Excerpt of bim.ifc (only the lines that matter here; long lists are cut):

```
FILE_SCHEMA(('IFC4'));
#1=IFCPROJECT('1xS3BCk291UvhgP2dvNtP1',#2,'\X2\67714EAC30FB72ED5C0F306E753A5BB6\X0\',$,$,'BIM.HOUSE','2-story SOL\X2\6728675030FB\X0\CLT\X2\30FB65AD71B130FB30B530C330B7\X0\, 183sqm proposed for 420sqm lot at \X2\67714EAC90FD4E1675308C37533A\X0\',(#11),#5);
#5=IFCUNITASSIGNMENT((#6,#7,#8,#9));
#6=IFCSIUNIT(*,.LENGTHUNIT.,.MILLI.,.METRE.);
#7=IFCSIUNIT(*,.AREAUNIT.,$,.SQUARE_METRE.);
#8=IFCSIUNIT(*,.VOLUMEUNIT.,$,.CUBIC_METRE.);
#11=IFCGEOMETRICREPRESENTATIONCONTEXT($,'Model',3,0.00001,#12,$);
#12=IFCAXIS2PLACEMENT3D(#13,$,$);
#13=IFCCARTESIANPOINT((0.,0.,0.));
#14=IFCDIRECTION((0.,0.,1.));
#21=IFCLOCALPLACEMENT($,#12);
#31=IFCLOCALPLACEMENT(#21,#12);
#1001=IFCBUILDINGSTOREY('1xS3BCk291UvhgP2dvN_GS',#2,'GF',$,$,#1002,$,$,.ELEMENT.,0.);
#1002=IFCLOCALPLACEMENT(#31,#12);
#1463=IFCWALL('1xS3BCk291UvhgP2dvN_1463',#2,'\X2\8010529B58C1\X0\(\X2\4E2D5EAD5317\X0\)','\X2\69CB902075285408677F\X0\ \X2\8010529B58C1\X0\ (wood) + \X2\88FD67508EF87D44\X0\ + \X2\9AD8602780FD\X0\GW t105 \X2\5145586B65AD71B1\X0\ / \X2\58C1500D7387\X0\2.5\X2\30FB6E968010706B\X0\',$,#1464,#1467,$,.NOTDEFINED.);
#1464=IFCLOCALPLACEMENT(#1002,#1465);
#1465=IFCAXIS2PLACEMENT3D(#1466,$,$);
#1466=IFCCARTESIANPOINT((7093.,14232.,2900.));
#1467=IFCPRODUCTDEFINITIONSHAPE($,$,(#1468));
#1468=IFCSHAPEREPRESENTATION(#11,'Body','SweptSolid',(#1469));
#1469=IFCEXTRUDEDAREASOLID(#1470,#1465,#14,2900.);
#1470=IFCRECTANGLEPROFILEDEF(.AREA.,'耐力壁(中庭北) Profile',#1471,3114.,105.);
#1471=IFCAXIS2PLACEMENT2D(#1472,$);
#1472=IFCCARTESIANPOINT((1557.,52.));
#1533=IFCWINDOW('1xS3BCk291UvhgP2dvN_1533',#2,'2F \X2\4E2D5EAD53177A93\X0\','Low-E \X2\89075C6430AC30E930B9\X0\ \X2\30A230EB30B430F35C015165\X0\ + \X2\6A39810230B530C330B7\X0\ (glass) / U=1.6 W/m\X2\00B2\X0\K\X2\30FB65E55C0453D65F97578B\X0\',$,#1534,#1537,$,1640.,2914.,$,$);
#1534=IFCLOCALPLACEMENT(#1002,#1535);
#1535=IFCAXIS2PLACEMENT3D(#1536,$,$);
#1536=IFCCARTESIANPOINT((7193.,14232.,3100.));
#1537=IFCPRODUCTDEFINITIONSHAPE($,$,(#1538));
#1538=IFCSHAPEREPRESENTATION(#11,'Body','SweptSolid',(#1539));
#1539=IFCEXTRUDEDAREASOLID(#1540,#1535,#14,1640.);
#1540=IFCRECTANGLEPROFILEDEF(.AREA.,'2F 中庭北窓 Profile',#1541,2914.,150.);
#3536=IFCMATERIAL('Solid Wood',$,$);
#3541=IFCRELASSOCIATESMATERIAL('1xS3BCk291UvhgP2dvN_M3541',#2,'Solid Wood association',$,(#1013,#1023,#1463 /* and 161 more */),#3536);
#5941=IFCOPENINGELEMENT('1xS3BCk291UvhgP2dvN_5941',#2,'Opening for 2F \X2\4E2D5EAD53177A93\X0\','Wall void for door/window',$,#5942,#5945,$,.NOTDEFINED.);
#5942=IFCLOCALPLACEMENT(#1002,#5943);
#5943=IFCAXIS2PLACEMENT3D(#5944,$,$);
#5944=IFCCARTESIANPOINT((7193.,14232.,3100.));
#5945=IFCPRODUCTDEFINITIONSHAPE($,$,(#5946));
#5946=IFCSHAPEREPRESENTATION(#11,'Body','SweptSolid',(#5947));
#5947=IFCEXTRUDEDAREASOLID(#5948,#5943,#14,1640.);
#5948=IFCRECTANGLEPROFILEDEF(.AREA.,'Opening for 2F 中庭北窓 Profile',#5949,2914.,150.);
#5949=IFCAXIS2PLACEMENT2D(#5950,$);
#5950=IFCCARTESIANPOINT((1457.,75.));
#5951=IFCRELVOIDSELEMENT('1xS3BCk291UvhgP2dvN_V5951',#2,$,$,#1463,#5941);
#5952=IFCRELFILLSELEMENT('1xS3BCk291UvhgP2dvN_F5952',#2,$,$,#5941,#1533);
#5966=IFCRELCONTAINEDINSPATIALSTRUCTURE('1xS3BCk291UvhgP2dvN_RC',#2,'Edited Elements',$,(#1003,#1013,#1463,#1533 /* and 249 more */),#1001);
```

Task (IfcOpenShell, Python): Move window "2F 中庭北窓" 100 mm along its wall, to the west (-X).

```python
import ifcopenshell
import ifcopenshell.api.geometry
import ifcopenshell.util.placement
import ifcopenshell.util.unit

model = ifcopenshell.open("bim.ifc")
unit_scale = ifcopenshell.util.unit.calculate_unit_scale(model)

window = model.by_guid("1xS3BCk291UvhgP2dvN_1533")
opening = window.FillsVoids[0].RelatingOpeningElement
wall = opening.VoidsElements[0].RelatingBuildingElement

wall_matrix = ifcopenshell.util.placement.get_local_placement(wall.ObjectPlacement)
shift = wall_matrix[:3, 0] * -0.1 / unit_scale
before = ifcopenshell.util.placement.get_local_placement(window.ObjectPlacement)[:3, 3].copy()

# The window is not placed relative to its opening, so move both.
for product in (opening, window):
    matrix = ifcopenshell.util.placement.get_local_placement(product.ObjectPlacement)
    matrix[:3, 3] += shift
    ifcopenshell.api.geometry.edit_object_placement(model, product=product, matrix=matrix, is_si=False)

after = ifcopenshell.util.placement.get_local_placement(window.ObjectPlacement)[:3, 3]
print("window moved by", (after - before).round(3) + 0.0)

model.write("bim_v2.ifc")
```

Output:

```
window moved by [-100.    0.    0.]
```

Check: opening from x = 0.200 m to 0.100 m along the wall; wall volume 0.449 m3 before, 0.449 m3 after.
